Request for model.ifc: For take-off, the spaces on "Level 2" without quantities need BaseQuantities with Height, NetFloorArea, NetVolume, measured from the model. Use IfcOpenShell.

First a look at what the model holds.

```python
import ifcopenshell
import ifcopenshell.util.element
import ifcopenshell.util.unit

model = ifcopenshell.open("model.ifc")
print(model.schema)
for unit_type in ("LENGTHUNIT", "AREAUNIT", "VOLUMEUNIT"):
    print(unit_type, ifcopenshell.util.unit.calculate_unit_scale(model, unit_type))
storey = next(s for s in model.by_type("IfcBuildingStorey") if s.Name == "Level 2")
spaces = [e for e in ifcopenshell.util.element.get_decomposition(storey) if e.is_a("IfcSpace")]
for e in sorted(spaces, key=lambda e: e.id()):
    print(e.id(), e.is_a(), e.Name, list(ifcopenshell.util.element.get_psets(e, qtos_only=True)), sep=" | ")
```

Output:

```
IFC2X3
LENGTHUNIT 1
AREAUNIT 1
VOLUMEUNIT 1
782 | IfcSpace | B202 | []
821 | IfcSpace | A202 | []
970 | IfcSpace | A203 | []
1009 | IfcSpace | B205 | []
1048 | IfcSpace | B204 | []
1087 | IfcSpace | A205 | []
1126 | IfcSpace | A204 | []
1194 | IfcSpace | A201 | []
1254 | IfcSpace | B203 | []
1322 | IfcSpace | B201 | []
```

```python
import ifcopenshell
import ifcopenshell.api.pset
import ifcopenshell.geom
import ifcopenshell.util.element
import ifcopenshell.util.shape
import ifcopenshell.util.unit

model = ifcopenshell.open("model.ifc")
unit_scale = ifcopenshell.util.unit.calculate_unit_scale(model)
area_scale = ifcopenshell.util.unit.calculate_unit_scale(model, "AREAUNIT")
volume_scale = ifcopenshell.util.unit.calculate_unit_scale(model, "VOLUMEUNIT")
settings = ifcopenshell.geom.settings()

storey = next(s for s in model.by_type("IfcBuildingStorey") if s.Name == "Level 2")
spaces = [e for e in ifcopenshell.util.element.get_decomposition(storey) if e.is_a("IfcSpace")]

for e in sorted(spaces, key=lambda e: e.id()):
    if ifcopenshell.util.element.get_psets(e, qtos_only=True, should_inherit=False):
        continue
    # Geometry comes back in metres, in the element's own axes.
    shape = ifcopenshell.geom.create_shape(settings, e)
    values = {
        "Height": ifcopenshell.util.shape.get_z(shape.geometry) / unit_scale,
        "NetFloorArea": ifcopenshell.util.shape.get_footprint_area(shape.geometry) / area_scale,
        "NetVolume": ifcopenshell.util.shape.get_volume(shape.geometry) / volume_scale,
    }
    qto = ifcopenshell.api.pset.add_qto(model, product=e, name="BaseQuantities")
    ifcopenshell.api.pset.edit_qto(model, qto=qto, properties=values)
    print(e.id(), {k: round(v, 3) for k, v in values.items()})

model.write("model_rev.ifc")
```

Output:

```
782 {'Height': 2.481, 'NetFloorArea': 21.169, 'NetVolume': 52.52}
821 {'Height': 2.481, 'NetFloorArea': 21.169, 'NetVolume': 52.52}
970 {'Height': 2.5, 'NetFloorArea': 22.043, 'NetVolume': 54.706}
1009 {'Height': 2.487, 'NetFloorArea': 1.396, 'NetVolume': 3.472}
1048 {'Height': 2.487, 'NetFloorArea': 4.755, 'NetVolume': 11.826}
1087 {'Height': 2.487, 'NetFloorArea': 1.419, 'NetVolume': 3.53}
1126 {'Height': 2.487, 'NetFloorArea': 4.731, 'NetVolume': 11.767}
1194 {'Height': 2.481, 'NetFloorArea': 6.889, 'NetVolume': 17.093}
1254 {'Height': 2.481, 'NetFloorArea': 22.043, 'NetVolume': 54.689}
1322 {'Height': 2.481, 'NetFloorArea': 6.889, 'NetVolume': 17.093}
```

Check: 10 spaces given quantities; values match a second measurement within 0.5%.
